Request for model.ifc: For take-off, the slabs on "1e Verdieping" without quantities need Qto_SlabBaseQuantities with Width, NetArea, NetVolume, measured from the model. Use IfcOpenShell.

First a look at what the model holds.

```python
import ifcopenshell
import ifcopenshell.util.element
import ifcopenshell.util.unit

model = ifcopenshell.open("model.ifc")
print(model.schema)
for unit_type in ("LENGTHUNIT", "AREAUNIT", "VOLUMEUNIT"):
    print(unit_type, ifcopenshell.util.unit.calculate_unit_scale(model, unit_type))
storey = next(s for s in model.by_type("IfcBuildingStorey") if s.Name == "1e Verdieping")
slabs = [e for e in ifcopenshell.util.element.get_decomposition(storey) if e.is_a("IfcSlab")]
for e in sorted(slabs, key=lambda e: e.id()):
    print(e.id(), e.is_a(), e.Name, list(ifcopenshell.util.element.get_psets(e, qtos_only=True)), sep=" | ")
```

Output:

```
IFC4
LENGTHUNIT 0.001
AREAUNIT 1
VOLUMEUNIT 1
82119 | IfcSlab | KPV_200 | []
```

```python
import ifcopenshell
import ifcopenshell.api.pset
import ifcopenshell.geom
import ifcopenshell.util.element
import ifcopenshell.util.shape
import ifcopenshell.util.unit

model = ifcopenshell.open("model.ifc")
unit_scale = ifcopenshell.util.unit.calculate_unit_scale(model)
area_scale = ifcopenshell.util.unit.calculate_unit_scale(model, "AREAUNIT")
volume_scale = ifcopenshell.util.unit.calculate_unit_scale(model, "VOLUMEUNIT")
settings = ifcopenshell.geom.settings()

storey = next(s for s in model.by_type("IfcBuildingStorey") if s.Name == "1e Verdieping")
slabs = [e for e in ifcopenshell.util.element.get_decomposition(storey) if e.is_a("IfcSlab")]

for e in sorted(slabs, key=lambda e: e.id()):
    if ifcopenshell.util.element.get_psets(e, qtos_only=True, should_inherit=False):
        continue
    # Geometry comes back in metres, in the element's own axes.
    shape = ifcopenshell.geom.create_shape(settings, e)
    values = {
        "Width": ifcopenshell.util.shape.get_z(shape.geometry) / unit_scale,
        "NetArea": ifcopenshell.util.shape.get_footprint_area(shape.geometry) / area_scale,
        "NetVolume": ifcopenshell.util.shape.get_volume(shape.geometry) / volume_scale,
    }
    qto = ifcopenshell.api.pset.add_qto(model, product=e, name="Qto_SlabBaseQuantities")
    ifcopenshell.api.pset.edit_qto(model, qto=qto, properties=values)
    print(e.id(), {k: round(v, 3) for k, v in values.items()})

model.write("model_rev.ifc")
```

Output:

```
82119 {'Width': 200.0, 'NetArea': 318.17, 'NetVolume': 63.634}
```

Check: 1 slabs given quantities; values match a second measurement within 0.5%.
